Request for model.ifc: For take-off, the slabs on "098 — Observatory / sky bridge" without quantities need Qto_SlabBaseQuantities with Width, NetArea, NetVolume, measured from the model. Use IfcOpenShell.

First a look at what the model holds.

```python
import ifcopenshell
import ifcopenshell.util.element
import ifcopenshell.util.unit

model = ifcopenshell.open("model.ifc")
print(model.schema)
for unit_type in ("LENGTHUNIT", "AREAUNIT", "VOLUMEUNIT"):
    print(unit_type, ifcopenshell.util.unit.calculate_unit_scale(model, unit_type))
storey = next(s for s in model.by_type("IfcBuildingStorey") if s.Name == "098 — Observatory / sky bridge")
slabs = [e for e in ifcopenshell.util.element.get_decomposition(storey) if e.is_a("IfcSlab")]
for e in sorted(slabs, key=lambda e: e.id()):
    print(e.id(), e.is_a(), e.Name, list(ifcopenshell.util.element.get_psets(e, qtos_only=True)), sep=" | ")
```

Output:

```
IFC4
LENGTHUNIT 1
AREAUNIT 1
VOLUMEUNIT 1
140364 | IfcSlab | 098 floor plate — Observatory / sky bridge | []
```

```python
import ifcopenshell
import ifcopenshell.api.pset
import ifcopenshell.geom
import ifcopenshell.util.element
import ifcopenshell.util.shape
import ifcopenshell.util.unit

model = ifcopenshell.open("model.ifc")
unit_scale = ifcopenshell.util.unit.calculate_unit_scale(model)
area_scale = ifcopenshell.util.unit.calculate_unit_scale(model, "AREAUNIT")
volume_scale = ifcopenshell.util.unit.calculate_unit_scale(model, "VOLUMEUNIT")
settings = ifcopenshell.geom.settings()

storey = next(s for s in model.by_type("IfcBuildingStorey") if s.Name == "098 — Observatory / sky bridge")
slabs = [e for e in ifcopenshell.util.element.get_decomposition(storey) if e.is_a("IfcSlab")]

for e in sorted(slabs, key=lambda e: e.id()):
    if ifcopenshell.util.element.get_psets(e, qtos_only=True, should_inherit=False):
        continue
    # Geometry comes back in metres, in the element's own axes.
    shape = ifcopenshell.geom.create_shape(settings, e)
    values = {
        "Width": ifcopenshell.util.shape.get_z(shape.geometry) / unit_scale,
        "NetArea": ifcopenshell.util.shape.get_footprint_area(shape.geometry) / area_scale,
        "NetVolume": ifcopenshell.util.shape.get_volume(shape.geometry) / volume_scale,
    }
    qto = ifcopenshell.api.pset.add_qto(model, product=e, name="Qto_SlabBaseQuantities")
    ifcopenshell.api.pset.edit_qto(model, qto=qto, properties=values)
    print(e.id(), {k: round(v, 3) for k, v in values.items()})

model.write("model-out.ifc")
```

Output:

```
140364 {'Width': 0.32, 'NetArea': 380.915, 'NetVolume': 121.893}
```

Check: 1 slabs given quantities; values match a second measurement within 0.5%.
